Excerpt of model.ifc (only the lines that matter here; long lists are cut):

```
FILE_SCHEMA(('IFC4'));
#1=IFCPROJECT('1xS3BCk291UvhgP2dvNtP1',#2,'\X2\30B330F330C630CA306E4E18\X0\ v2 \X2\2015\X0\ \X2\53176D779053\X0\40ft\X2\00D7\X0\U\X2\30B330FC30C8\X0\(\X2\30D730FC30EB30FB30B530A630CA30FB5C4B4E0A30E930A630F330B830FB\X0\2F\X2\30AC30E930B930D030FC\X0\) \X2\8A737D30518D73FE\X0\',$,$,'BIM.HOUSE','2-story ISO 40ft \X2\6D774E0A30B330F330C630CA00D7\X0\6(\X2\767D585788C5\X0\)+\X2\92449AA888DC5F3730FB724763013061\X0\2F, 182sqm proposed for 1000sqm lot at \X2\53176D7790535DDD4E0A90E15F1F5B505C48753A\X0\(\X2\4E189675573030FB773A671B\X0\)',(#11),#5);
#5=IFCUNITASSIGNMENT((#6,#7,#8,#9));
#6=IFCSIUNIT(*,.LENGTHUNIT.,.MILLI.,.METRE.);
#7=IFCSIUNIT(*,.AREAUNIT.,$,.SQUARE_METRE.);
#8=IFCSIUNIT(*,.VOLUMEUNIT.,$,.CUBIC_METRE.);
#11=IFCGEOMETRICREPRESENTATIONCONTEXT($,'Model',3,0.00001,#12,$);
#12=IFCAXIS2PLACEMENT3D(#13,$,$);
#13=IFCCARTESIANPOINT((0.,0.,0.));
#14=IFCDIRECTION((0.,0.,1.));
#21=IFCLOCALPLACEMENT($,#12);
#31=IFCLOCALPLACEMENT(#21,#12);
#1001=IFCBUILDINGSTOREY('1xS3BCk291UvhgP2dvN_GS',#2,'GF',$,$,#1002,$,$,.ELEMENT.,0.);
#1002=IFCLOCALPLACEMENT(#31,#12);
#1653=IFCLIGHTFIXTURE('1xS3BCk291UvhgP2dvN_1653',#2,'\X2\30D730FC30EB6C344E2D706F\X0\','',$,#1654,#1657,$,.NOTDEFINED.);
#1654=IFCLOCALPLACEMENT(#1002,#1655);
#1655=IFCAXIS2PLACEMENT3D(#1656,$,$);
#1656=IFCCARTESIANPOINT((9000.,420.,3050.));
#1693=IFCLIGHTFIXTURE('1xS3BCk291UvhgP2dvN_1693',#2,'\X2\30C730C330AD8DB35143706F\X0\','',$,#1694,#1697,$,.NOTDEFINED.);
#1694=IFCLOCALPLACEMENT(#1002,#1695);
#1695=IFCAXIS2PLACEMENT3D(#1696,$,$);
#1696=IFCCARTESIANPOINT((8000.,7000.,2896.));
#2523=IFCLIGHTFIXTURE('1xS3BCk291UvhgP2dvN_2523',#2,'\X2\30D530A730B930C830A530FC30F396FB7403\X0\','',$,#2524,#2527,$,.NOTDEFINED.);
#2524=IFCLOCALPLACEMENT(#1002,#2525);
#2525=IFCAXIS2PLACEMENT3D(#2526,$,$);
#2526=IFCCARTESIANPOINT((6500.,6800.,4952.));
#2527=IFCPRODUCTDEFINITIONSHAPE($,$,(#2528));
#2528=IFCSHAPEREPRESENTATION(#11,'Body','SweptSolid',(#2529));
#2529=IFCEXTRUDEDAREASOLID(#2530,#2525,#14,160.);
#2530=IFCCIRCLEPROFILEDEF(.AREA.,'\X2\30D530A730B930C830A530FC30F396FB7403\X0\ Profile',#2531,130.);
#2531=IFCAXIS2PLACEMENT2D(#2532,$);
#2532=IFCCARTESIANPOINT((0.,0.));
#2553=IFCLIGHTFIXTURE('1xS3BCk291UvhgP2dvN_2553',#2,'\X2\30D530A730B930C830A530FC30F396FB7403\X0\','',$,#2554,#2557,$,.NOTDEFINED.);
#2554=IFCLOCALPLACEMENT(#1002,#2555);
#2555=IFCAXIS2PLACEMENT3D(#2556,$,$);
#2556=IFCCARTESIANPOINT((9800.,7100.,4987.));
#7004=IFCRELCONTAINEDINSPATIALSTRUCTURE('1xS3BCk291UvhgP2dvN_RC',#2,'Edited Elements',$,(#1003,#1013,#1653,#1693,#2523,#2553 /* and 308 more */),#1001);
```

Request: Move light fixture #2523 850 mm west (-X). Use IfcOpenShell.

```python
import ifcopenshell
import ifcopenshell.api.geometry
import ifcopenshell.util.placement
import ifcopenshell.util.unit

model = ifcopenshell.open("model.ifc")
unit_scale = ifcopenshell.util.unit.calculate_unit_scale(model)

item = model.by_id(2523)
matrix = ifcopenshell.util.placement.get_local_placement(item.ObjectPlacement)
matrix[0, 3] -= 0.85 / unit_scale
ifcopenshell.api.geometry.edit_object_placement(model, product=item, matrix=matrix, is_si=False)

print(ifcopenshell.util.placement.get_local_placement(item.ObjectPlacement).round(3) + 0.0)

model.write("model_edited.ifc")
```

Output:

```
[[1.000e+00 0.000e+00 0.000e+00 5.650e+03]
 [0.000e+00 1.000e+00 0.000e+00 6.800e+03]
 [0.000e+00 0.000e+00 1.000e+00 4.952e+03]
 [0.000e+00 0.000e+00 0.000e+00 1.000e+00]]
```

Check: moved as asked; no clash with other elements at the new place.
